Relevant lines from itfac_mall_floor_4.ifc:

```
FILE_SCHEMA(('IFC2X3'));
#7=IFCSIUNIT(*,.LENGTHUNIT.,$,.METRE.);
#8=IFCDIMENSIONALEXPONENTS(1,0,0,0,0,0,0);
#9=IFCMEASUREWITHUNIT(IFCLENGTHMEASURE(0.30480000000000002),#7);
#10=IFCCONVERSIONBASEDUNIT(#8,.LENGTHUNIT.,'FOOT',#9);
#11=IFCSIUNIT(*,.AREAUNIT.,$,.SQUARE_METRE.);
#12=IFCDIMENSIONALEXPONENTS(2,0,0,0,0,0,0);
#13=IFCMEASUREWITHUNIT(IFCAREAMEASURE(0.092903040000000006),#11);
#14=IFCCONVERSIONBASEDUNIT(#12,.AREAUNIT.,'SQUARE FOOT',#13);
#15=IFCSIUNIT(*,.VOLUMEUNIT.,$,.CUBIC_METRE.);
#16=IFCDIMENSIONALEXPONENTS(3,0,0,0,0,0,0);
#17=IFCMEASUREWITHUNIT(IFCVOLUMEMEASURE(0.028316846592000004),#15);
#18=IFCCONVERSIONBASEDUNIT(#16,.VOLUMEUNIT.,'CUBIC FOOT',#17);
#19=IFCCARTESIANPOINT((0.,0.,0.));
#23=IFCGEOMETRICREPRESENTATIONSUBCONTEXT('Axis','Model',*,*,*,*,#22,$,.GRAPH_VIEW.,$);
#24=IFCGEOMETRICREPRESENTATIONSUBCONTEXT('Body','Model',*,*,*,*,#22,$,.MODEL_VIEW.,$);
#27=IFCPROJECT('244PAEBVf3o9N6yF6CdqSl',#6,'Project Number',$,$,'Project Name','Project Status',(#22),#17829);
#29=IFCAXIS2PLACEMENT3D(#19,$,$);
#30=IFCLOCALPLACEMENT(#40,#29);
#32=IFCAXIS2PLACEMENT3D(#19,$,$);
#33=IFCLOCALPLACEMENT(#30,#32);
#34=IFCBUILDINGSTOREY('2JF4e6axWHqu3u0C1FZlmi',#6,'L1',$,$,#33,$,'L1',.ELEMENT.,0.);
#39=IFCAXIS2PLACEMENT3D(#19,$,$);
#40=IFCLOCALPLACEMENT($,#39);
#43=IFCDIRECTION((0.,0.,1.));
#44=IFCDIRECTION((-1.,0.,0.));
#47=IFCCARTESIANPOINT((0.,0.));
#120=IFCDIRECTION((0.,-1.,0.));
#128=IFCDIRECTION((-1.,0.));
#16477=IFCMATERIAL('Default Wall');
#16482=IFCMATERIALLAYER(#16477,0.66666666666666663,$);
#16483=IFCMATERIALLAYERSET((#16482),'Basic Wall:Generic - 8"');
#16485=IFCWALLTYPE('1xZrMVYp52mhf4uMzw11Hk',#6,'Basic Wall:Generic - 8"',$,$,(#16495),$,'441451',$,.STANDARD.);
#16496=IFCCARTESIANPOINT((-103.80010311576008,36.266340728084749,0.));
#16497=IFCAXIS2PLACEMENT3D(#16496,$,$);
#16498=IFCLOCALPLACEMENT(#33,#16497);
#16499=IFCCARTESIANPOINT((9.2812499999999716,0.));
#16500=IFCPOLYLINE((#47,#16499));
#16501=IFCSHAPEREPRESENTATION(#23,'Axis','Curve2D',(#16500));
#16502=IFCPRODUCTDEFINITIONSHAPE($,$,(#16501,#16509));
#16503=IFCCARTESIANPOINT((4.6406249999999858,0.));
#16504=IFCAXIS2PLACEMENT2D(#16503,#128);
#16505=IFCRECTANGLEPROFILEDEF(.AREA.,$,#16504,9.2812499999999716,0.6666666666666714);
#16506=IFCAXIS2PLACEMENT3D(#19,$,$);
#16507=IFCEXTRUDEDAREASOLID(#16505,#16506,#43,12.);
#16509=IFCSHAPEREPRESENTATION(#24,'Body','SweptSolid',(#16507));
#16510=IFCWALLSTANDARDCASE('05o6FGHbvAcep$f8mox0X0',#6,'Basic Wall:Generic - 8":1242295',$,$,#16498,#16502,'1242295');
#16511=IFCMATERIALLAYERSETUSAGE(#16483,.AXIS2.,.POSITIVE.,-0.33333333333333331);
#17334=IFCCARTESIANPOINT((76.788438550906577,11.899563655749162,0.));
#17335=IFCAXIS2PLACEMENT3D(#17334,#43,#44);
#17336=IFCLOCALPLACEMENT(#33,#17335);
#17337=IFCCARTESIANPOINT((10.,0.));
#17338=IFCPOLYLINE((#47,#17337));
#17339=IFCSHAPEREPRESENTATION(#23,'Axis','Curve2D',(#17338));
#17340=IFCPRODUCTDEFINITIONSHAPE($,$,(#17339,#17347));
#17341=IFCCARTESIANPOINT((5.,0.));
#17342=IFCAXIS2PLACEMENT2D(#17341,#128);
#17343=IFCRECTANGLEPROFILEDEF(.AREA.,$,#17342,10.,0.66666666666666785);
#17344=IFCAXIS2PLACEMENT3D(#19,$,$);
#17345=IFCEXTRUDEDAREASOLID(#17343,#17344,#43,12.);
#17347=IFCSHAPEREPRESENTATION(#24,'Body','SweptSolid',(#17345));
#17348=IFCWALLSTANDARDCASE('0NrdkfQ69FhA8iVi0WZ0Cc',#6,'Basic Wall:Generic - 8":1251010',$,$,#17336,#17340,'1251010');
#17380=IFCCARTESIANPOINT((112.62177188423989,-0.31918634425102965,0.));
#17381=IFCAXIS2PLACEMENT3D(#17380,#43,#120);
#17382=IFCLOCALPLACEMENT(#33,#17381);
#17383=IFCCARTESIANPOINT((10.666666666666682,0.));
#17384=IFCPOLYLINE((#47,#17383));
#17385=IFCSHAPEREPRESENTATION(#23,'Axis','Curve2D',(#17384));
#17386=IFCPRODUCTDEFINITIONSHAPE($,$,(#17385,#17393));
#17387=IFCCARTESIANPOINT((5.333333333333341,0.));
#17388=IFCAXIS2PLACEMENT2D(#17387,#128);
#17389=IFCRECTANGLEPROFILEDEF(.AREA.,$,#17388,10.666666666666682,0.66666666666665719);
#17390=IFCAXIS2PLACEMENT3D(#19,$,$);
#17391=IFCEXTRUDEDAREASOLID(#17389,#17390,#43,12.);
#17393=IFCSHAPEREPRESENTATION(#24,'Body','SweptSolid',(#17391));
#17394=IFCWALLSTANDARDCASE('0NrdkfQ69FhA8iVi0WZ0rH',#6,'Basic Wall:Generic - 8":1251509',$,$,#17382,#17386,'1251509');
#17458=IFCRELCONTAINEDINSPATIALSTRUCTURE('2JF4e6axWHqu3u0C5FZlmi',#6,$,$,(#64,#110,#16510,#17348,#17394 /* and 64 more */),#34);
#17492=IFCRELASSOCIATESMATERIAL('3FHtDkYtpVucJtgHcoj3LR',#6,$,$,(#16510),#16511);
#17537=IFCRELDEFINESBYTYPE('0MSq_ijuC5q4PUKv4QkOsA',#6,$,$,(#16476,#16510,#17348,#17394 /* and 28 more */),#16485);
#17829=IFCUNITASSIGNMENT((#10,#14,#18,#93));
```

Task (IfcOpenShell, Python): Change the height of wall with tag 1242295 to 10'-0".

```python
import ifcopenshell
import ifcopenshell.geom
import ifcopenshell.util.representation
import ifcopenshell.util.shape
import ifcopenshell.util.unit

model = ifcopenshell.open("itfac_mall_floor_4.ifc")
unit_scale = ifcopenshell.util.unit.calculate_unit_scale(model)
settings = ifcopenshell.geom.settings()


def volume(element):
    """Net volume in cubic metres, openings subtracted."""
    shape = ifcopenshell.geom.create_shape(settings, element)
    return ifcopenshell.util.shape.get_volume(shape.geometry)


wall = model.by_guid("05o6FGHbvAcep$f8mox0X0")
before = volume(wall)

body = ifcopenshell.util.representation.get_representation(wall, "Model", "Body")
solid = body.Items[0]
old_height = solid.Depth
solid.Depth = 120 * 0.0254 / unit_scale
after = volume(wall)

print(f"height {old_height:g} -> {solid.Depth:g}, volume {before:.3f} -> {after:.3f} m3")

model.write("itfac_mall_floor_4_updated.ifc")
```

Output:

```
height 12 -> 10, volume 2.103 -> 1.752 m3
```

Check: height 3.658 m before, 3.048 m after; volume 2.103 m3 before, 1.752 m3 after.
